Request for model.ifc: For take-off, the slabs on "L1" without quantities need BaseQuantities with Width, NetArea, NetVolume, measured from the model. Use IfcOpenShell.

First a look at what the model holds.

```python
import ifcopenshell
import ifcopenshell.util.element
import ifcopenshell.util.unit

model = ifcopenshell.open("model.ifc")
print(model.schema)
for unit_type in ("LENGTHUNIT", "AREAUNIT", "VOLUMEUNIT"):
    print(unit_type, ifcopenshell.util.unit.calculate_unit_scale(model, unit_type))
storey = next(s for s in model.by_type("IfcBuildingStorey") if s.Name == "L1")
slabs = [e for e in ifcopenshell.util.element.get_decomposition(storey) if e.is_a("IfcSlab")]
for e in sorted(slabs, key=lambda e: e.id()):
    print(e.id(), e.is_a(), e.Name, list(ifcopenshell.util.element.get_psets(e, qtos_only=True)), sep=" | ")
```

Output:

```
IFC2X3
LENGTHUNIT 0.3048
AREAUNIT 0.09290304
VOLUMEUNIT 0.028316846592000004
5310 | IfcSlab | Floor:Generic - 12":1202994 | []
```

```python
import ifcopenshell
import ifcopenshell.api.pset
import ifcopenshell.geom
import ifcopenshell.util.element
import ifcopenshell.util.shape
import ifcopenshell.util.unit

model = ifcopenshell.open("model.ifc")
unit_scale = ifcopenshell.util.unit.calculate_unit_scale(model)
area_scale = ifcopenshell.util.unit.calculate_unit_scale(model, "AREAUNIT")
volume_scale = ifcopenshell.util.unit.calculate_unit_scale(model, "VOLUMEUNIT")
settings = ifcopenshell.geom.settings()

storey = next(s for s in model.by_type("IfcBuildingStorey") if s.Name == "L1")
slabs = [e for e in ifcopenshell.util.element.get_decomposition(storey) if e.is_a("IfcSlab")]

for e in sorted(slabs, key=lambda e: e.id()):
    if ifcopenshell.util.element.get_psets(e, qtos_only=True, should_inherit=False):
        continue
    # Geometry comes back in metres, in the element's own axes.
    shape = ifcopenshell.geom.create_shape(settings, e)
    values = {
        "Width": ifcopenshell.util.shape.get_z(shape.geometry) / unit_scale,
        "NetArea": ifcopenshell.util.shape.get_footprint_area(shape.geometry) / area_scale,
        "NetVolume": ifcopenshell.util.shape.get_volume(shape.geometry) / volume_scale,
    }
    qto = ifcopenshell.api.pset.add_qto(model, product=e, name="BaseQuantities")
    ifcopenshell.api.pset.edit_qto(model, qto=qto, properties=values)
    print(e.id(), {k: round(v, 3) for k, v in values.items()})

model.write("model_updated.ifc")
```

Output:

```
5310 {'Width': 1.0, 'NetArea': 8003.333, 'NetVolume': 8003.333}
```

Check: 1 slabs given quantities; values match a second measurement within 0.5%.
